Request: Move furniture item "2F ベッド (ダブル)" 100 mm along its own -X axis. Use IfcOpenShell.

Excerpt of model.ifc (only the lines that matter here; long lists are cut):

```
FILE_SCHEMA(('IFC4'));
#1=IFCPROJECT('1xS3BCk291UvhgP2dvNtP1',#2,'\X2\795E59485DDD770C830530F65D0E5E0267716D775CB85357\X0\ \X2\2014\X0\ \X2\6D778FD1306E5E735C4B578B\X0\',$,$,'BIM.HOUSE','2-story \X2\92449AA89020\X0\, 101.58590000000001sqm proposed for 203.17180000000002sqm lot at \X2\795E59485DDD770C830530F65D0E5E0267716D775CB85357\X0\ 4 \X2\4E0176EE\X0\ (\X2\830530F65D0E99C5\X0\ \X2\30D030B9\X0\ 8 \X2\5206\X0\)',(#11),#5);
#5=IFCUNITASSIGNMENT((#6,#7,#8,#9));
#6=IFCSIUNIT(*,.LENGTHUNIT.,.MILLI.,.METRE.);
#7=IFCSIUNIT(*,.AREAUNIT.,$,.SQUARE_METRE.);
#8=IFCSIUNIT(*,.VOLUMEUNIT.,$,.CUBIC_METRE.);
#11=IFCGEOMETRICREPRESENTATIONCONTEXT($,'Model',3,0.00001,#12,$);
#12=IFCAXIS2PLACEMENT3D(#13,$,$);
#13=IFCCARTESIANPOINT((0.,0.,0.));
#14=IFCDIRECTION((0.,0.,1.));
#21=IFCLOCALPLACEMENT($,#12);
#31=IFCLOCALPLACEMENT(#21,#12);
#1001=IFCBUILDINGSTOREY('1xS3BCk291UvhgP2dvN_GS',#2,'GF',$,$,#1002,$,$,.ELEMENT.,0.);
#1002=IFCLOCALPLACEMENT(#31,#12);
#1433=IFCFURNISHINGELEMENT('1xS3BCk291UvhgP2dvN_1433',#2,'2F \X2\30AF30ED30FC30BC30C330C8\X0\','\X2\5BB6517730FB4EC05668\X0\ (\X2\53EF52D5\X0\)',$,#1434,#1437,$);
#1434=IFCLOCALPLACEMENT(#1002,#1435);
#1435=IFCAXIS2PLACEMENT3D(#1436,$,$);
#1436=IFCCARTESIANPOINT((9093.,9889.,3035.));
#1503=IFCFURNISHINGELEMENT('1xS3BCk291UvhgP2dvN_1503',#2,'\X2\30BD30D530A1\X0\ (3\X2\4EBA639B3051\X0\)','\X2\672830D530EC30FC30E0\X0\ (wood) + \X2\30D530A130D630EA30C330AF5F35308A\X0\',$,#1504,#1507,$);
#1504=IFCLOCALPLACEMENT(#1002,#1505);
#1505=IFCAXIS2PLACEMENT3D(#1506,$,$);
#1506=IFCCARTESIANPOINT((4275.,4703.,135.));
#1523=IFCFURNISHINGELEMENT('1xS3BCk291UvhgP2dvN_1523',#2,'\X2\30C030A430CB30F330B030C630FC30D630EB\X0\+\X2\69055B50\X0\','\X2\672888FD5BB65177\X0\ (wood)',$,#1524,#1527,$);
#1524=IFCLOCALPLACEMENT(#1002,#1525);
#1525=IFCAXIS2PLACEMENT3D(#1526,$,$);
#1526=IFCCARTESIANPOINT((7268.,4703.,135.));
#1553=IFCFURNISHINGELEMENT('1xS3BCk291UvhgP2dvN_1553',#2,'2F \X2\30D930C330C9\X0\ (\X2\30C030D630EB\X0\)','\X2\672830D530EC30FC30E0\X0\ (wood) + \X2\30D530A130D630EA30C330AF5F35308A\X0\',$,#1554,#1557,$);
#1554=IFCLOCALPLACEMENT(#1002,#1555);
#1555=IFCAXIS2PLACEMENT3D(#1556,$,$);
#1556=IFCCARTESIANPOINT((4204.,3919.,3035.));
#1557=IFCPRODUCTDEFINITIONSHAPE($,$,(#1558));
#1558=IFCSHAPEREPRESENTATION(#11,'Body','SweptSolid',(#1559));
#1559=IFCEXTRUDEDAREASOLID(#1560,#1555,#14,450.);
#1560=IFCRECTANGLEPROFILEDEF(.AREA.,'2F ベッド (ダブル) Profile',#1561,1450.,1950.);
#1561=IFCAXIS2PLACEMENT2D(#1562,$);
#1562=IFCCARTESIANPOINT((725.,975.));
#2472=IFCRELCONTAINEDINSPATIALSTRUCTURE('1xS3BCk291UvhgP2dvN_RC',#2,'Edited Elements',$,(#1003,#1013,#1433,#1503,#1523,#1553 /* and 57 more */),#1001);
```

```python
import ifcopenshell
import ifcopenshell.api.geometry
import ifcopenshell.util.placement

model = ifcopenshell.open("model.ifc")

item = model.by_guid("1xS3BCk291UvhgP2dvN_1553")
matrix = ifcopenshell.util.placement.get_local_placement(item.ObjectPlacement)
matrix[:3, 3] -= matrix[:3, 0] * 100.0
ifcopenshell.api.geometry.edit_object_placement(model, product=item, matrix=matrix, is_si=False)

print(ifcopenshell.util.placement.get_local_placement(item.ObjectPlacement).round(3) + 0.0)

model.write("model_updated.ifc")
```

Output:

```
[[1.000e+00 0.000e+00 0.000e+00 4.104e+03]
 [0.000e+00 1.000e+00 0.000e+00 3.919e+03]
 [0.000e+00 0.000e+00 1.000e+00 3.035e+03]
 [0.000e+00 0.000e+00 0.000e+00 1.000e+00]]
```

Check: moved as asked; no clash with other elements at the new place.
